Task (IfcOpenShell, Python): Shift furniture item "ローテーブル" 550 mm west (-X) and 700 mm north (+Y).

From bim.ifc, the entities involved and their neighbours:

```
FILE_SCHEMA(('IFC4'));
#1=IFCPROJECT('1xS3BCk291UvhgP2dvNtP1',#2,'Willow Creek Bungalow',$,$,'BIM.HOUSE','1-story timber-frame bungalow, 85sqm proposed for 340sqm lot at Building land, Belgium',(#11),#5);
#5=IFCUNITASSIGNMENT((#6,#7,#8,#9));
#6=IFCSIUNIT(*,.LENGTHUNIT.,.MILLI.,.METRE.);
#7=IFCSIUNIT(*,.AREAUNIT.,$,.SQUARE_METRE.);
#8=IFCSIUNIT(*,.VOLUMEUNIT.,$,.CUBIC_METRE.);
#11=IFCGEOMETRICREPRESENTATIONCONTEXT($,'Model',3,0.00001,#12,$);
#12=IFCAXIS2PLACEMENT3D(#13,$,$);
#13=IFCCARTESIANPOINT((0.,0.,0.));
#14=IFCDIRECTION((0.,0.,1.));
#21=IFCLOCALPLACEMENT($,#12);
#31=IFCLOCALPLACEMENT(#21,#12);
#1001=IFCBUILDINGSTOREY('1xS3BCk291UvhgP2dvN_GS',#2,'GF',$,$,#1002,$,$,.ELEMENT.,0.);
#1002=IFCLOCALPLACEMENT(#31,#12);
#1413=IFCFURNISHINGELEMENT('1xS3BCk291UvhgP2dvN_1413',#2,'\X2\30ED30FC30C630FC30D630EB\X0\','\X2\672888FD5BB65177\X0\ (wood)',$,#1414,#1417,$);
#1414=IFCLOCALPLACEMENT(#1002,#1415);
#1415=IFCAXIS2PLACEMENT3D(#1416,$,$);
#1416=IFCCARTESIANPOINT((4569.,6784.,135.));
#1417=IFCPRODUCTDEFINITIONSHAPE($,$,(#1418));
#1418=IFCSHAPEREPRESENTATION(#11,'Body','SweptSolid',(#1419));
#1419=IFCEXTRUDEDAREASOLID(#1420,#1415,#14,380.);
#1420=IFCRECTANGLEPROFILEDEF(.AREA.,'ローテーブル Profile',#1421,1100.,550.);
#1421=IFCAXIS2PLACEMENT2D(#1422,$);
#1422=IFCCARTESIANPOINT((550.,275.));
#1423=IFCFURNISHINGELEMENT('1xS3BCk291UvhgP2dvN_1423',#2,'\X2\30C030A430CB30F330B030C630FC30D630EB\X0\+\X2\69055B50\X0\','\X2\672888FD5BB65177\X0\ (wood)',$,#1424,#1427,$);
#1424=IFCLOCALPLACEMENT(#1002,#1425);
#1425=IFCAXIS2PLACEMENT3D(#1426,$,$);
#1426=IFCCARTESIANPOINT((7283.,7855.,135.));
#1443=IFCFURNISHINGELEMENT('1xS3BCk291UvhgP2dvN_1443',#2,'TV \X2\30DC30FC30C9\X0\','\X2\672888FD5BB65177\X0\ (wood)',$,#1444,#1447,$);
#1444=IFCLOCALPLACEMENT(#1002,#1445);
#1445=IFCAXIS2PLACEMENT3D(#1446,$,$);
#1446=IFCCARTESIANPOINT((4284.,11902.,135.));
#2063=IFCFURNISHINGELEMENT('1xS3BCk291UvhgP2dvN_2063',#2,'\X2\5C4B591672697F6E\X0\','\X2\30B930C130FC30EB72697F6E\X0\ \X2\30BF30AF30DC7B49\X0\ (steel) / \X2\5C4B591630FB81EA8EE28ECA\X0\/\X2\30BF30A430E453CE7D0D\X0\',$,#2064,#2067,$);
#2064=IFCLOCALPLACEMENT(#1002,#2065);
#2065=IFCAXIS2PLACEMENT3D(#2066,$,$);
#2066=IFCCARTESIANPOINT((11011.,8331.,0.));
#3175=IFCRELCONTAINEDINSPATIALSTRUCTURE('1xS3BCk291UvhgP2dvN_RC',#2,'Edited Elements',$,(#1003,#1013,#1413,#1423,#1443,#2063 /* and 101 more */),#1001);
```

```python
import ifcopenshell
import ifcopenshell.api.geometry
import ifcopenshell.util.placement
import ifcopenshell.util.unit

model = ifcopenshell.open("bim.ifc")
unit_scale = ifcopenshell.util.unit.calculate_unit_scale(model)

item = model.by_id(1413)
matrix = ifcopenshell.util.placement.get_local_placement(item.ObjectPlacement)
matrix[0, 3] -= 0.55 / unit_scale
matrix[1, 3] += 0.7 / unit_scale
ifcopenshell.api.geometry.edit_object_placement(model, product=item, matrix=matrix, is_si=False)

print(ifcopenshell.util.placement.get_local_placement(item.ObjectPlacement).round(3) + 0.0)

model.write("bim_v2.ifc")
```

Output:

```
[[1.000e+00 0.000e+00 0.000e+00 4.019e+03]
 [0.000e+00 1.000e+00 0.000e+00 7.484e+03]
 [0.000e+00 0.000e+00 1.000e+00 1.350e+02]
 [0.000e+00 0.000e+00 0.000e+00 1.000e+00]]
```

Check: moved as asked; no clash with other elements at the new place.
